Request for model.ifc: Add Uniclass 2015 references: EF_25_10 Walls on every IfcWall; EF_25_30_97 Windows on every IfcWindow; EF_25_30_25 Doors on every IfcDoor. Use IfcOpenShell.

First a look at what the model holds.

```python
import ifcopenshell

model = ifcopenshell.open("model.ifc")
print(model.schema)
print("classifications:", [c.Name for c in model.by_type("IfcClassification")])
for ifc_class in ("IfcDoor", "IfcRoof", "IfcStair", "IfcWall", "IfcWindow"):
    print(ifc_class, len(model.by_type(ifc_class)))
```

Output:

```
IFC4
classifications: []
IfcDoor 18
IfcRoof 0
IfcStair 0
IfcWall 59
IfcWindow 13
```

```python
import ifcopenshell
import ifcopenshell.api.classification

model = ifcopenshell.open("model.ifc")

system = ifcopenshell.api.classification.add_classification(model, classification="Uniclass 2015")

codes = {
    "IfcWall": ("EF_25_10", "Walls"),
    "IfcWindow": ("EF_25_30_97", "Windows"),
    "IfcDoor": ("EF_25_30_25", "Doors"),
}
for ifc_class, (code, name) in codes.items():
    products = model.by_type(ifc_class)
    ifcopenshell.api.classification.add_reference(
        model, products=products, classification=system, identification=code, name=name
    )
    print(code, len(products))

model.write("model_updated.ifc")
```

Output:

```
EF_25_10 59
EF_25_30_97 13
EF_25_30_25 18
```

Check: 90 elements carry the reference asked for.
